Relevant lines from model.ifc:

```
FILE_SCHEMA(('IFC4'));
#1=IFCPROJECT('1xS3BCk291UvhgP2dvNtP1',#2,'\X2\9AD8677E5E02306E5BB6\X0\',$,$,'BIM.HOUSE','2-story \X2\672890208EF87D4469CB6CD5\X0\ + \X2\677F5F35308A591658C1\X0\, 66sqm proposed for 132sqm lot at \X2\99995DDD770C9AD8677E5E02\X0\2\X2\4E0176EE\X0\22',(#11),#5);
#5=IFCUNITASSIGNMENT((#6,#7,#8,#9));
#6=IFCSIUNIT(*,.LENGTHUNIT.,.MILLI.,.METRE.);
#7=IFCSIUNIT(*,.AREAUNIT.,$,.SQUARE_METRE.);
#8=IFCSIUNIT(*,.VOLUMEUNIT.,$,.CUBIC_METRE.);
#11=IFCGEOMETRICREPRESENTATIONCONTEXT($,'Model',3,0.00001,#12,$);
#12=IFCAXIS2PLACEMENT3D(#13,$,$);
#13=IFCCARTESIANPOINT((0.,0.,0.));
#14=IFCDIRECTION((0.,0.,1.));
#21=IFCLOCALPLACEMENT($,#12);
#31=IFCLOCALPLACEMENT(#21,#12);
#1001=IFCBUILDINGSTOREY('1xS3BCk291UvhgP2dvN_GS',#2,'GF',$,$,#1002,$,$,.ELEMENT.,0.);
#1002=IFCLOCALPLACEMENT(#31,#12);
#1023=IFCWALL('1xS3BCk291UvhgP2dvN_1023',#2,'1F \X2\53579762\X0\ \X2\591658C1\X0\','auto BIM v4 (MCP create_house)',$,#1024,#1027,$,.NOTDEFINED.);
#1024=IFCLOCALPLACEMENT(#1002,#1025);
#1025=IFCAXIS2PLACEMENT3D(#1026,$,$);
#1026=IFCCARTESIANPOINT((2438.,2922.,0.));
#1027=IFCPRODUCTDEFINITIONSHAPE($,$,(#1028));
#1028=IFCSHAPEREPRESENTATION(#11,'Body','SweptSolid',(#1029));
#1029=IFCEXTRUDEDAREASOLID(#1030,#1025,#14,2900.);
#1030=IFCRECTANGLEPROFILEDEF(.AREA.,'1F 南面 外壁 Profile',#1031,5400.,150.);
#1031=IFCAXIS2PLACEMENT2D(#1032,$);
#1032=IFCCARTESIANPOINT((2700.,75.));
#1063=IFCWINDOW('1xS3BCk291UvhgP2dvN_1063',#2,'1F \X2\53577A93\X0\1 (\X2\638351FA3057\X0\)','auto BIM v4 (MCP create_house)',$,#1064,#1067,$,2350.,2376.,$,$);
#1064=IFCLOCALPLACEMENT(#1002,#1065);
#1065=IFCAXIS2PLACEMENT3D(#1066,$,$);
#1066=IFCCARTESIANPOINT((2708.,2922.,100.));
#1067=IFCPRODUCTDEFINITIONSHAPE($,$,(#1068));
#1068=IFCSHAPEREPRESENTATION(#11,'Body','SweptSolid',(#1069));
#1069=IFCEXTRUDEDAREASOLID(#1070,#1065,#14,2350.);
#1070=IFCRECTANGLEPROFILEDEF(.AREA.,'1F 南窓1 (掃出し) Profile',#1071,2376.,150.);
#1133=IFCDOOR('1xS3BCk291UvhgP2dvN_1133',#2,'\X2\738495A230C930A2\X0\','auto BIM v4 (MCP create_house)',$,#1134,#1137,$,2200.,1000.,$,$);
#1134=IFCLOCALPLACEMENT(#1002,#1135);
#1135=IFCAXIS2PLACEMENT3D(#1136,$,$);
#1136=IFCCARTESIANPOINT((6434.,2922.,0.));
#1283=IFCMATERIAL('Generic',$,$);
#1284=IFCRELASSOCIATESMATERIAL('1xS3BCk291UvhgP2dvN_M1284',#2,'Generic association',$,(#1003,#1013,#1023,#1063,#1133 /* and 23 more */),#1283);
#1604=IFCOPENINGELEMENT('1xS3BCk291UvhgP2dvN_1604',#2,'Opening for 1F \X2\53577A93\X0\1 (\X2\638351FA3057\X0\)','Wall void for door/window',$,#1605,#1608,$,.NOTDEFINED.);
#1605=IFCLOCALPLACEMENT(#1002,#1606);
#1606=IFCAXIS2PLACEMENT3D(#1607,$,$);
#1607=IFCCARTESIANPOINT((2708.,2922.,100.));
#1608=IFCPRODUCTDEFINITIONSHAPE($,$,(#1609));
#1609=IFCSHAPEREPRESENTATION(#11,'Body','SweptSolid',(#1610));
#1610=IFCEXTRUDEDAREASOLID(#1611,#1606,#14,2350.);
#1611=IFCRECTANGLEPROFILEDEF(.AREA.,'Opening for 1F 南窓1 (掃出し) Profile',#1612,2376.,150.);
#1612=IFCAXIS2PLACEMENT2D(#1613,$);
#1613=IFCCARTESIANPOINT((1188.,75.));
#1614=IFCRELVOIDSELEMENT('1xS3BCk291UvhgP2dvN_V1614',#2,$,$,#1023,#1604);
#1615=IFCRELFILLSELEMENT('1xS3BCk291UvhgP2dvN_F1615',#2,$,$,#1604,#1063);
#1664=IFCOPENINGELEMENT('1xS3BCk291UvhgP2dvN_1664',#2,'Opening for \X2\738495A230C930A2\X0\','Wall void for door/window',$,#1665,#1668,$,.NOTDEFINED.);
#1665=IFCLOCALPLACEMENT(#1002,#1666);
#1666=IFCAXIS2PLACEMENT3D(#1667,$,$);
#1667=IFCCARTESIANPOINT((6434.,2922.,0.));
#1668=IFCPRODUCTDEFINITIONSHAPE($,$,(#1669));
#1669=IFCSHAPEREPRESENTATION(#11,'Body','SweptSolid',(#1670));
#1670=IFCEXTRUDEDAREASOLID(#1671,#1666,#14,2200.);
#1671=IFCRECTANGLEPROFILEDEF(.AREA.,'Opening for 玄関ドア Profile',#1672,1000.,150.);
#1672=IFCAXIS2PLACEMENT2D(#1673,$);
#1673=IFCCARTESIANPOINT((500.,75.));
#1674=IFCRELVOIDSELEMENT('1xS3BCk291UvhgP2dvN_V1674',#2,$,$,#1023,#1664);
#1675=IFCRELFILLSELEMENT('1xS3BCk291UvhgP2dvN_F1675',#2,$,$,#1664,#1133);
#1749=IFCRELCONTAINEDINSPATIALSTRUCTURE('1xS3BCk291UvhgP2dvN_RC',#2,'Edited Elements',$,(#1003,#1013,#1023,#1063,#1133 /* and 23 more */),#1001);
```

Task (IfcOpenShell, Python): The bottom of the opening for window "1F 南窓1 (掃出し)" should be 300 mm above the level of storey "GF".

```python
import numpy as np
import ifcopenshell
import ifcopenshell.api.geometry
import ifcopenshell.geom
import ifcopenshell.util.element
import ifcopenshell.util.placement
import ifcopenshell.util.shape
import ifcopenshell.util.unit

model = ifcopenshell.open("model.ifc")
unit_scale = ifcopenshell.util.unit.calculate_unit_scale(model)

window = model.by_guid("1xS3BCk291UvhgP2dvN_1063")
opening = window.FillsVoids[0].RelatingOpeningElement
storey = ifcopenshell.util.element.get_container(window, ifc_class="IfcBuildingStorey")
level = ifcopenshell.util.placement.get_local_placement(storey.ObjectPlacement)[2, 3]

# The opening's origin need not be at the sill, so measure its lowest point.
shape = ifcopenshell.geom.create_shape(ifcopenshell.geom.settings(), opening)
bottom = ifcopenshell.util.shape.get_shape_bottom_elevation(shape, shape.geometry) / unit_scale
dz = level + 300.0 - bottom

shift = np.array([0.0, 0.0, dz])
# The window is not placed relative to its opening, so move both.
for product in (opening, window):
    matrix = ifcopenshell.util.placement.get_local_placement(product.ObjectPlacement)
    matrix[:3, 3] += shift
    ifcopenshell.api.geometry.edit_object_placement(model, product=product, matrix=matrix, is_si=False)

print(f"moved by {dz * unit_scale:+.3f} m")

model.write("model_updated.ifc")
```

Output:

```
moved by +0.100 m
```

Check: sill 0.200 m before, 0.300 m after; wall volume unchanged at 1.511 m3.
